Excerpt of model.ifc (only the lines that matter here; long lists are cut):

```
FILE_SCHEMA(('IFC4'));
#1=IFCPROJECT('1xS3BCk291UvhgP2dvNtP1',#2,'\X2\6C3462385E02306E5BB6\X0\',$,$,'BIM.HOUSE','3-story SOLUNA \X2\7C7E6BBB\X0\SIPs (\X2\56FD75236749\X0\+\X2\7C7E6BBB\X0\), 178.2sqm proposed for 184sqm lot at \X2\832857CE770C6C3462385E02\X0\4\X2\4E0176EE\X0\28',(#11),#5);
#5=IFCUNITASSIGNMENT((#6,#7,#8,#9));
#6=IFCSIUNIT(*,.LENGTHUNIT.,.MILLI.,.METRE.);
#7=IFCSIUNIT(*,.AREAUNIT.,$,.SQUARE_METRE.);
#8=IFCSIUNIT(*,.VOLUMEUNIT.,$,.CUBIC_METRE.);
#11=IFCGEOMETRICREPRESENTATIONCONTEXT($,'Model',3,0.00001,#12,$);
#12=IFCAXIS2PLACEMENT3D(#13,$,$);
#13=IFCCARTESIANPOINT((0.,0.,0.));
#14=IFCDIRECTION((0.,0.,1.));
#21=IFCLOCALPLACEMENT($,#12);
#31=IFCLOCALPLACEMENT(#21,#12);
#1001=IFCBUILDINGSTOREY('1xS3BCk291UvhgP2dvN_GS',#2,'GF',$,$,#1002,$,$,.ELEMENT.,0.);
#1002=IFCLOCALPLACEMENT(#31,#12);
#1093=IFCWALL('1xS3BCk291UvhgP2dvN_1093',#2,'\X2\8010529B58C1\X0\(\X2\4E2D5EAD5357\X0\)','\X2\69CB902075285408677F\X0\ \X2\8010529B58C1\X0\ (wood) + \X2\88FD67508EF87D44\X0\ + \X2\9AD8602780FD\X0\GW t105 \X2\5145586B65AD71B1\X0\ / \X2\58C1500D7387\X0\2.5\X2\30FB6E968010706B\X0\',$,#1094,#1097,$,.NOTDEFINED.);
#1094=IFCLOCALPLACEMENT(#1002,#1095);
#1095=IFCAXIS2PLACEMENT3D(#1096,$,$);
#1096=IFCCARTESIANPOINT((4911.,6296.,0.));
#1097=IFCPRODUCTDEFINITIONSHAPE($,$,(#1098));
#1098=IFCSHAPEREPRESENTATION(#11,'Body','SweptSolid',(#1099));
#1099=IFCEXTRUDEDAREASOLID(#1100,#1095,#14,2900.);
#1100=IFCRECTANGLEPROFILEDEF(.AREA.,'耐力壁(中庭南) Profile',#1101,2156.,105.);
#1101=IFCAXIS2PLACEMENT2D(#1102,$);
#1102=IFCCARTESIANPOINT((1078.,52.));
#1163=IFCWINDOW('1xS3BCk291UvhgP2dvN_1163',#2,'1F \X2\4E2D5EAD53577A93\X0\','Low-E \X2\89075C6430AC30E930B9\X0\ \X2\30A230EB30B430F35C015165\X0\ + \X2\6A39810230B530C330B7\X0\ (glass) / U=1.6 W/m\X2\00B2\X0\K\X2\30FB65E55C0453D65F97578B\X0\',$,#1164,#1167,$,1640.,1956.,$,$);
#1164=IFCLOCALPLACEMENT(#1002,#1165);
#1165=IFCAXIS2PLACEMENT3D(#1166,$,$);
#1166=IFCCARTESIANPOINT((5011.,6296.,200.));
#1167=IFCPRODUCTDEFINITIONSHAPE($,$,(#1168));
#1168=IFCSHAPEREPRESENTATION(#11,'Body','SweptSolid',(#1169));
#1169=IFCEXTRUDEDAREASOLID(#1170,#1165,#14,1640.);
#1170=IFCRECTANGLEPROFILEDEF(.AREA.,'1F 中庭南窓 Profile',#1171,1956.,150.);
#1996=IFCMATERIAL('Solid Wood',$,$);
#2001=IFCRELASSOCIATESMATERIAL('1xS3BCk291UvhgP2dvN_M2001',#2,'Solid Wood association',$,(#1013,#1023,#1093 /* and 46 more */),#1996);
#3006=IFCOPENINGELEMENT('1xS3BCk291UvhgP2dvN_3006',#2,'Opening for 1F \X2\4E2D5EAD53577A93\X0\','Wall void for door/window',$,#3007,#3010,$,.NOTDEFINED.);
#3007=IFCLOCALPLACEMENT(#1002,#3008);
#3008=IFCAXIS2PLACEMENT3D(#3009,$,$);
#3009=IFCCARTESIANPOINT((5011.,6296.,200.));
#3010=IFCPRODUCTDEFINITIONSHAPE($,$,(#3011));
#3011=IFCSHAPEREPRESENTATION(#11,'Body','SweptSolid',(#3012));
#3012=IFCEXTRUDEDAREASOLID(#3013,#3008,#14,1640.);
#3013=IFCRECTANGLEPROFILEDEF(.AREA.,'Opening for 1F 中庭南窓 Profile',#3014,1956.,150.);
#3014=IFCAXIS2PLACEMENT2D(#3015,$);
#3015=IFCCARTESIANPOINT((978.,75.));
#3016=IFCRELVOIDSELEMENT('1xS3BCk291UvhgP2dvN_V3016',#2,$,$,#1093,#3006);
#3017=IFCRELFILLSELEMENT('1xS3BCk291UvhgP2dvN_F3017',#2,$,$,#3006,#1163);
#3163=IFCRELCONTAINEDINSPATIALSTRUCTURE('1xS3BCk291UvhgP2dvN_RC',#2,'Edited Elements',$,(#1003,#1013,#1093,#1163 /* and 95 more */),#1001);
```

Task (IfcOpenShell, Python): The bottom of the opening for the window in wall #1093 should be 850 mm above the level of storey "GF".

```python
import numpy as np
import ifcopenshell
import ifcopenshell.api.geometry
import ifcopenshell.geom
import ifcopenshell.util.element
import ifcopenshell.util.placement
import ifcopenshell.util.shape
import ifcopenshell.util.unit

model = ifcopenshell.open("model.ifc")
unit_scale = ifcopenshell.util.unit.calculate_unit_scale(model)

window = model.by_guid("1xS3BCk291UvhgP2dvN_1163")
opening = window.FillsVoids[0].RelatingOpeningElement
storey = ifcopenshell.util.element.get_container(window, ifc_class="IfcBuildingStorey")
level = ifcopenshell.util.placement.get_local_placement(storey.ObjectPlacement)[2, 3]

# The opening's origin need not be at the sill, so measure its lowest point.
shape = ifcopenshell.geom.create_shape(ifcopenshell.geom.settings(), opening)
bottom = ifcopenshell.util.shape.get_shape_bottom_elevation(shape, shape.geometry) / unit_scale
dz = level + 0.85 / unit_scale - bottom

shift = np.array([0.0, 0.0, dz])
# The window is not placed relative to its opening, so move both.
for product in (opening, window):
    matrix = ifcopenshell.util.placement.get_local_placement(product.ObjectPlacement)
    matrix[:3, 3] += shift
    ifcopenshell.api.geometry.edit_object_placement(model, product=product, matrix=matrix, is_si=False)

print(f"moved by {dz * unit_scale:+.3f} m")

model.write("model_v2.ifc")
```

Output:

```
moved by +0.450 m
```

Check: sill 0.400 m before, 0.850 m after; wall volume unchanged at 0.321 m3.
